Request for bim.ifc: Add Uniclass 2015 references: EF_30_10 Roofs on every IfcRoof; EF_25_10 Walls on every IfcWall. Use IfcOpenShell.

First a look at what the model holds.

```python
import ifcopenshell

model = ifcopenshell.open("bim.ifc")
print(model.schema)
print("classifications:", [c.Name for c in model.by_type("IfcClassification")])
for ifc_class in ("IfcDoor", "IfcRoof", "IfcStair", "IfcWall", "IfcWindow"):
    print(ifc_class, len(model.by_type(ifc_class)))
```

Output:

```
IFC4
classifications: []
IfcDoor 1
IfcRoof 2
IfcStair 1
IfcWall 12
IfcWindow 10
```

```python
import ifcopenshell
import ifcopenshell.api.classification

model = ifcopenshell.open("bim.ifc")

system = ifcopenshell.api.classification.add_classification(model, classification="Uniclass 2015")

codes = {
    "IfcRoof": ("EF_30_10", "Roofs"),
    "IfcWall": ("EF_25_10", "Walls"),
}
for ifc_class, (code, name) in codes.items():
    products = model.by_type(ifc_class)
    ifcopenshell.api.classification.add_reference(
        model, products=products, classification=system, identification=code, name=name
    )
    print(code, len(products))

model.write("bim-out.ifc")
```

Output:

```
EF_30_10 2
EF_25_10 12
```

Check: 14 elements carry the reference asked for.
